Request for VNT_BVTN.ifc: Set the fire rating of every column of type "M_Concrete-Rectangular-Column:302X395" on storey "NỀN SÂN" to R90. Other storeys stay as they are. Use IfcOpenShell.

First a look at what the model holds.

```python
import ifcopenshell
import ifcopenshell.util.element

model = ifcopenshell.open("VNT_BVTN.ifc")
print(model.schema)
storey = next(s for s in model.by_type("IfcBuildingStorey") if s.Name == "NỀN SÂN")
columns = [e for e in ifcopenshell.util.element.get_decomposition(storey) if e.is_a("IfcColumn")]
seen = {}
for e in columns:
    element_type = ifcopenshell.util.element.get_type(e)
    key = (element_type.Name if element_type != e and element_type else None, ifcopenshell.util.element.get_pset(e, "Pset_ColumnCommon", "FireRating"))
    seen[key] = seen.get(key, 0) + 1
for (name, value), count in sorted(seen.items(), key=str):
    print(count, "x", name, "|", value)
```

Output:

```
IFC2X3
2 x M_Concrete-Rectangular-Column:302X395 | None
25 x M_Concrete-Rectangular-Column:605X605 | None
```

```python
import ifcopenshell
import ifcopenshell.api.pset
import ifcopenshell.util.element

model = ifcopenshell.open("VNT_BVTN.ifc")

storey = next(s for s in model.by_type("IfcBuildingStorey") if s.Name == "NỀN SÂN")
columns = [e for e in ifcopenshell.util.element.get_decomposition(storey) if e.is_a("IfcColumn")]

count = 0
for e in columns:
    element_type = ifcopenshell.util.element.get_type(e)
    if element_type in (None, e) or element_type.Name != "M_Concrete-Rectangular-Column:302X395":
        continue
    # add_pset returns the element's existing set when there is one.
    pset = ifcopenshell.api.pset.add_pset(model, product=e, name="Pset_ColumnCommon")
    ifcopenshell.api.pset.edit_pset(model, pset=pset, properties={"FireRating": "R90"})
    count += 1

print(count, "columns updated")

model.write("VNT_BVTN_edited.ifc")
```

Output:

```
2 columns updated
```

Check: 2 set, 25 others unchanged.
